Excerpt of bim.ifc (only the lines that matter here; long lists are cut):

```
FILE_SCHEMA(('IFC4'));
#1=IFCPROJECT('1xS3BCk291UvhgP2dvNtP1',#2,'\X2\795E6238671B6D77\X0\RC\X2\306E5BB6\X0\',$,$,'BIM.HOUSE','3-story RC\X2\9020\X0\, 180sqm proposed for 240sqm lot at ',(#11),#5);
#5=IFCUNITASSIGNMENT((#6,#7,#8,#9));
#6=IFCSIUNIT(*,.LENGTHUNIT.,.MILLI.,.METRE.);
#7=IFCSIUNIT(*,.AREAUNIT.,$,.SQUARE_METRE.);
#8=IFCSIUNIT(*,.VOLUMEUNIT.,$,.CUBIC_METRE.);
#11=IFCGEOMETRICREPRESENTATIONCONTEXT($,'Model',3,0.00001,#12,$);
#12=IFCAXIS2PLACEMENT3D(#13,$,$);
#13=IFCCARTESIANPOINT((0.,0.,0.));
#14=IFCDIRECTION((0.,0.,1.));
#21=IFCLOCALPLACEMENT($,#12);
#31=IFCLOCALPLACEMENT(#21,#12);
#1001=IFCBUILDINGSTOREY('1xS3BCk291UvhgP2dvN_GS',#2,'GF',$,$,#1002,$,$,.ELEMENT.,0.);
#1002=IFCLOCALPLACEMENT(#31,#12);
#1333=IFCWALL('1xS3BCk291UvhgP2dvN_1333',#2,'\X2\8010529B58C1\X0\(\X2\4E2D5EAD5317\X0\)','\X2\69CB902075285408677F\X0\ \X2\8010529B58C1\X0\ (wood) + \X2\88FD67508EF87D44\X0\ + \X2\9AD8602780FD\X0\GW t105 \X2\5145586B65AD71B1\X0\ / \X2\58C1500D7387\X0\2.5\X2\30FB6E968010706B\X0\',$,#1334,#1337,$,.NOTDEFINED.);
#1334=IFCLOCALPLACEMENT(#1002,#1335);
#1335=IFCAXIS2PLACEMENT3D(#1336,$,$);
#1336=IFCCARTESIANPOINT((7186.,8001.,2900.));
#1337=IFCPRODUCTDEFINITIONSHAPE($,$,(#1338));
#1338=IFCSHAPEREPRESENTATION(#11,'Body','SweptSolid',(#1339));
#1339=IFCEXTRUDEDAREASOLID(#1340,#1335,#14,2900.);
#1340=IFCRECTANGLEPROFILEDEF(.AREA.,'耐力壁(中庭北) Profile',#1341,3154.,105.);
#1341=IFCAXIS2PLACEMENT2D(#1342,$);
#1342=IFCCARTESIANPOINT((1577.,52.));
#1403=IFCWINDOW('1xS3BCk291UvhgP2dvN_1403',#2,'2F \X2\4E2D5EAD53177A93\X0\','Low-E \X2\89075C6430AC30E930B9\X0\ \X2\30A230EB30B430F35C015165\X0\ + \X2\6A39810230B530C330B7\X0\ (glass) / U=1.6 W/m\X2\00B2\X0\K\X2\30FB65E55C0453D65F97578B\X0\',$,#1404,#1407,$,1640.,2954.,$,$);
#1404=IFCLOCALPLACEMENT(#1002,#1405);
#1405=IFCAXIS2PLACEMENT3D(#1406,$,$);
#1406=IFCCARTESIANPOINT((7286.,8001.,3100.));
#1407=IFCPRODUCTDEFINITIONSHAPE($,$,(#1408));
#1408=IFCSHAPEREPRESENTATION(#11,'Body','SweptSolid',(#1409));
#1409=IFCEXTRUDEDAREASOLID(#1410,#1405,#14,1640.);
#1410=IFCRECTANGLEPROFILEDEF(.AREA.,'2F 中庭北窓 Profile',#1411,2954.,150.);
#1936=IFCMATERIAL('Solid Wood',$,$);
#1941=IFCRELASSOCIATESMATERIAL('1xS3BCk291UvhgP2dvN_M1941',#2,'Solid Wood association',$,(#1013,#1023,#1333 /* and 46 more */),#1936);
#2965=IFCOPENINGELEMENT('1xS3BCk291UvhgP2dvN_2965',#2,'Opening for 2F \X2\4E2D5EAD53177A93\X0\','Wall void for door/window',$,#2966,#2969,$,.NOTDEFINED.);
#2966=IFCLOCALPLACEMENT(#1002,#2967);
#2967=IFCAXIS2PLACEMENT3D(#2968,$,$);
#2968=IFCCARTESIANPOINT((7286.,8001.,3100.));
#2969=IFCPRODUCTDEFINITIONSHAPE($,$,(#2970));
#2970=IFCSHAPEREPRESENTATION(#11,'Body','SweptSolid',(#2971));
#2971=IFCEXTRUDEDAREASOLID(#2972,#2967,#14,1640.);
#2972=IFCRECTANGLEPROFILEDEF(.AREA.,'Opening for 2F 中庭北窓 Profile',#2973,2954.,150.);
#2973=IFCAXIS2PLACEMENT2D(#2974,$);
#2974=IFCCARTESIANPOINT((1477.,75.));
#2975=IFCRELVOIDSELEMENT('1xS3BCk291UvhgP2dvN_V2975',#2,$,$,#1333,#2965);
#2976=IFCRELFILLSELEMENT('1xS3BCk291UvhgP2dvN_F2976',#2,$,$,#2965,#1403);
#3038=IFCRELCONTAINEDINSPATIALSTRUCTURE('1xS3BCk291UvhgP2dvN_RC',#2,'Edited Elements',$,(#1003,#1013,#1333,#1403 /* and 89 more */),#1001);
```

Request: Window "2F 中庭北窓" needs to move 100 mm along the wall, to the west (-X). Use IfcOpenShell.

```python
import ifcopenshell
import ifcopenshell.api.geometry
import ifcopenshell.util.placement

model = ifcopenshell.open("bim.ifc")

window = model.by_guid("1xS3BCk291UvhgP2dvN_1403")
opening = window.FillsVoids[0].RelatingOpeningElement
wall = opening.VoidsElements[0].RelatingBuildingElement

wall_matrix = ifcopenshell.util.placement.get_local_placement(wall.ObjectPlacement)
shift = wall_matrix[:3, 0] * -100.0
before = ifcopenshell.util.placement.get_local_placement(window.ObjectPlacement)[:3, 3].copy()

# The window is not placed relative to its opening, so move both.
for product in (opening, window):
    matrix = ifcopenshell.util.placement.get_local_placement(product.ObjectPlacement)
    matrix[:3, 3] += shift
    ifcopenshell.api.geometry.edit_object_placement(model, product=product, matrix=matrix, is_si=False)

after = ifcopenshell.util.placement.get_local_placement(window.ObjectPlacement)[:3, 3]
print("window moved by", (after - before).round(3) + 0.0)

model.write("bim_rev.ifc")
```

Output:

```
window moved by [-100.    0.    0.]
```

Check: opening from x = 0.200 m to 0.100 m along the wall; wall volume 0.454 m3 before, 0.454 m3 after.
